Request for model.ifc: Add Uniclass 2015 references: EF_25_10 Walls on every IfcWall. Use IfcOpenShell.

First a look at what the model holds.

```python
import ifcopenshell

model = ifcopenshell.open("model.ifc")
print(model.schema)
print("classifications:", [c.Name for c in model.by_type("IfcClassification")])
for ifc_class in ("IfcDoor", "IfcRoof", "IfcStair", "IfcWall", "IfcWindow"):
    print(ifc_class, len(model.by_type(ifc_class)))
```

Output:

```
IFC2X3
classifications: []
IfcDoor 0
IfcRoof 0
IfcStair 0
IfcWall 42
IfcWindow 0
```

```python
import ifcopenshell
import ifcopenshell.api.classification

model = ifcopenshell.open("model.ifc")

# IFC2X3 requires Source and Edition and has no link from the project to the system.
system = model.create_entity("IfcClassification", Source="NBS", Edition="2015", Name="Uniclass 2015")

codes = {
    "IfcWall": ("EF_25_10", "Walls"),
}
for ifc_class, (code, name) in codes.items():
    products = model.by_type(ifc_class)
    ifcopenshell.api.classification.add_reference(
        model, products=products, classification=system, identification=code, name=name
    )
    print(code, len(products))

model.write("model_rev.ifc")
```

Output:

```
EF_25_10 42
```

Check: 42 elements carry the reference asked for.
